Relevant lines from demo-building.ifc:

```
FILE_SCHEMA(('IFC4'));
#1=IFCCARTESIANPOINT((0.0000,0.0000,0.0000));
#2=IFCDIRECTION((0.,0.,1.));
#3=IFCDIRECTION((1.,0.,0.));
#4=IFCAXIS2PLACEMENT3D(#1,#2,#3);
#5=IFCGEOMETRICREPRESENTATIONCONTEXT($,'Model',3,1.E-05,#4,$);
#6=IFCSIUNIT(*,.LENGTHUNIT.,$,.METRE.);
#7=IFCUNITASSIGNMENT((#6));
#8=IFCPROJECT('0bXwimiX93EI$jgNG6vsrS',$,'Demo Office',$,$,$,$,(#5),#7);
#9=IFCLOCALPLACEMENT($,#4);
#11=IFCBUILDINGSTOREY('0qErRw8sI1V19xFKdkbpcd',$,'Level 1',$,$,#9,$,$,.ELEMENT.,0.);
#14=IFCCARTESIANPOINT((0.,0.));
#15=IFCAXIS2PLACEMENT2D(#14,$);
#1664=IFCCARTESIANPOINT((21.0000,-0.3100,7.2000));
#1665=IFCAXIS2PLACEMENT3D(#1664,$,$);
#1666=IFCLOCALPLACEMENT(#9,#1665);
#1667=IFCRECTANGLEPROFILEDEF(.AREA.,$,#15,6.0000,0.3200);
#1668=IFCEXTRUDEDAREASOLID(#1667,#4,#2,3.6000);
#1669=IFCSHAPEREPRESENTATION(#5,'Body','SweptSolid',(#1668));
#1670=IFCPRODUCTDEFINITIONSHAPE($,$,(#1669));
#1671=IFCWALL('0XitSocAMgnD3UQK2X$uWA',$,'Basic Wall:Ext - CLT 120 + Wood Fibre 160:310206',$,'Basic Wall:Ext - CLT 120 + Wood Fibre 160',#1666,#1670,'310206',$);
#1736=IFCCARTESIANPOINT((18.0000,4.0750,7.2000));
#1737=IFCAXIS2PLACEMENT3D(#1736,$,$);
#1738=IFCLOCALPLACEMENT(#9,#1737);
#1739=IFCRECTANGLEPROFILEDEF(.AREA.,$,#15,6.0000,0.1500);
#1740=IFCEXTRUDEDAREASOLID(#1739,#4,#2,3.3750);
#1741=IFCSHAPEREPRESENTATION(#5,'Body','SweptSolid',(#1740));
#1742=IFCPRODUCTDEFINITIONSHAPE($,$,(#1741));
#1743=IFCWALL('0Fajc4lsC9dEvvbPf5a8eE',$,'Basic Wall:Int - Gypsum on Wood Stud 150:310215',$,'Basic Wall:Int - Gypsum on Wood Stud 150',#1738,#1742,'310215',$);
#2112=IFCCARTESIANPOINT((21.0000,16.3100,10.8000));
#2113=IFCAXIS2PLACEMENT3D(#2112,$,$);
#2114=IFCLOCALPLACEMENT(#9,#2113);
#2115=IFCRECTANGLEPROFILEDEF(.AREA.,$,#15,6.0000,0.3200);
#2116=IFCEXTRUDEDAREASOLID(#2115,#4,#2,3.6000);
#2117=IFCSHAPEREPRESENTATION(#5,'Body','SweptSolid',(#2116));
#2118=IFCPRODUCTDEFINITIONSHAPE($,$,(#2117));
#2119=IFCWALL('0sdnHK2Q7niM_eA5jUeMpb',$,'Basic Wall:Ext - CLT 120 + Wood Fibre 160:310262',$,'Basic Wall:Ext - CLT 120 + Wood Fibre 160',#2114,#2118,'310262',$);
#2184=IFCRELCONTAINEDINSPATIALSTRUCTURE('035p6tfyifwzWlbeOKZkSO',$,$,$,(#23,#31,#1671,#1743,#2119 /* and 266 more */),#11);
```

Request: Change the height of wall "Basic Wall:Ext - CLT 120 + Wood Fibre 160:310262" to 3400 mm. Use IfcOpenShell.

```python
import ifcopenshell
import ifcopenshell.geom
import ifcopenshell.util.shape

model = ifcopenshell.open("demo-building.ifc")
settings = ifcopenshell.geom.settings()


def volume(element):
    """Net volume in cubic metres, openings subtracted."""
    shape = ifcopenshell.geom.create_shape(settings, element)
    return ifcopenshell.util.shape.get_volume(shape.geometry)


wall = model.by_guid("0sdnHK2Q7niM_eA5jUeMpb")
before = volume(wall)

body = next(r for r in wall.Representation.Representations if r.RepresentationIdentifier == "Body")
solid = body.Items[0]
old_height = solid.Depth
solid.Depth = 3.4
after = volume(wall)

print(f"height {old_height:g} -> {solid.Depth:g}, volume {before:.3f} -> {after:.3f} m3")

model.write("demo-building_v2.ifc")
```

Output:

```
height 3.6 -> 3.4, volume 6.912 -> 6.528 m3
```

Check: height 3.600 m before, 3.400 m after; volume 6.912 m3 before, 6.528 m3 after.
